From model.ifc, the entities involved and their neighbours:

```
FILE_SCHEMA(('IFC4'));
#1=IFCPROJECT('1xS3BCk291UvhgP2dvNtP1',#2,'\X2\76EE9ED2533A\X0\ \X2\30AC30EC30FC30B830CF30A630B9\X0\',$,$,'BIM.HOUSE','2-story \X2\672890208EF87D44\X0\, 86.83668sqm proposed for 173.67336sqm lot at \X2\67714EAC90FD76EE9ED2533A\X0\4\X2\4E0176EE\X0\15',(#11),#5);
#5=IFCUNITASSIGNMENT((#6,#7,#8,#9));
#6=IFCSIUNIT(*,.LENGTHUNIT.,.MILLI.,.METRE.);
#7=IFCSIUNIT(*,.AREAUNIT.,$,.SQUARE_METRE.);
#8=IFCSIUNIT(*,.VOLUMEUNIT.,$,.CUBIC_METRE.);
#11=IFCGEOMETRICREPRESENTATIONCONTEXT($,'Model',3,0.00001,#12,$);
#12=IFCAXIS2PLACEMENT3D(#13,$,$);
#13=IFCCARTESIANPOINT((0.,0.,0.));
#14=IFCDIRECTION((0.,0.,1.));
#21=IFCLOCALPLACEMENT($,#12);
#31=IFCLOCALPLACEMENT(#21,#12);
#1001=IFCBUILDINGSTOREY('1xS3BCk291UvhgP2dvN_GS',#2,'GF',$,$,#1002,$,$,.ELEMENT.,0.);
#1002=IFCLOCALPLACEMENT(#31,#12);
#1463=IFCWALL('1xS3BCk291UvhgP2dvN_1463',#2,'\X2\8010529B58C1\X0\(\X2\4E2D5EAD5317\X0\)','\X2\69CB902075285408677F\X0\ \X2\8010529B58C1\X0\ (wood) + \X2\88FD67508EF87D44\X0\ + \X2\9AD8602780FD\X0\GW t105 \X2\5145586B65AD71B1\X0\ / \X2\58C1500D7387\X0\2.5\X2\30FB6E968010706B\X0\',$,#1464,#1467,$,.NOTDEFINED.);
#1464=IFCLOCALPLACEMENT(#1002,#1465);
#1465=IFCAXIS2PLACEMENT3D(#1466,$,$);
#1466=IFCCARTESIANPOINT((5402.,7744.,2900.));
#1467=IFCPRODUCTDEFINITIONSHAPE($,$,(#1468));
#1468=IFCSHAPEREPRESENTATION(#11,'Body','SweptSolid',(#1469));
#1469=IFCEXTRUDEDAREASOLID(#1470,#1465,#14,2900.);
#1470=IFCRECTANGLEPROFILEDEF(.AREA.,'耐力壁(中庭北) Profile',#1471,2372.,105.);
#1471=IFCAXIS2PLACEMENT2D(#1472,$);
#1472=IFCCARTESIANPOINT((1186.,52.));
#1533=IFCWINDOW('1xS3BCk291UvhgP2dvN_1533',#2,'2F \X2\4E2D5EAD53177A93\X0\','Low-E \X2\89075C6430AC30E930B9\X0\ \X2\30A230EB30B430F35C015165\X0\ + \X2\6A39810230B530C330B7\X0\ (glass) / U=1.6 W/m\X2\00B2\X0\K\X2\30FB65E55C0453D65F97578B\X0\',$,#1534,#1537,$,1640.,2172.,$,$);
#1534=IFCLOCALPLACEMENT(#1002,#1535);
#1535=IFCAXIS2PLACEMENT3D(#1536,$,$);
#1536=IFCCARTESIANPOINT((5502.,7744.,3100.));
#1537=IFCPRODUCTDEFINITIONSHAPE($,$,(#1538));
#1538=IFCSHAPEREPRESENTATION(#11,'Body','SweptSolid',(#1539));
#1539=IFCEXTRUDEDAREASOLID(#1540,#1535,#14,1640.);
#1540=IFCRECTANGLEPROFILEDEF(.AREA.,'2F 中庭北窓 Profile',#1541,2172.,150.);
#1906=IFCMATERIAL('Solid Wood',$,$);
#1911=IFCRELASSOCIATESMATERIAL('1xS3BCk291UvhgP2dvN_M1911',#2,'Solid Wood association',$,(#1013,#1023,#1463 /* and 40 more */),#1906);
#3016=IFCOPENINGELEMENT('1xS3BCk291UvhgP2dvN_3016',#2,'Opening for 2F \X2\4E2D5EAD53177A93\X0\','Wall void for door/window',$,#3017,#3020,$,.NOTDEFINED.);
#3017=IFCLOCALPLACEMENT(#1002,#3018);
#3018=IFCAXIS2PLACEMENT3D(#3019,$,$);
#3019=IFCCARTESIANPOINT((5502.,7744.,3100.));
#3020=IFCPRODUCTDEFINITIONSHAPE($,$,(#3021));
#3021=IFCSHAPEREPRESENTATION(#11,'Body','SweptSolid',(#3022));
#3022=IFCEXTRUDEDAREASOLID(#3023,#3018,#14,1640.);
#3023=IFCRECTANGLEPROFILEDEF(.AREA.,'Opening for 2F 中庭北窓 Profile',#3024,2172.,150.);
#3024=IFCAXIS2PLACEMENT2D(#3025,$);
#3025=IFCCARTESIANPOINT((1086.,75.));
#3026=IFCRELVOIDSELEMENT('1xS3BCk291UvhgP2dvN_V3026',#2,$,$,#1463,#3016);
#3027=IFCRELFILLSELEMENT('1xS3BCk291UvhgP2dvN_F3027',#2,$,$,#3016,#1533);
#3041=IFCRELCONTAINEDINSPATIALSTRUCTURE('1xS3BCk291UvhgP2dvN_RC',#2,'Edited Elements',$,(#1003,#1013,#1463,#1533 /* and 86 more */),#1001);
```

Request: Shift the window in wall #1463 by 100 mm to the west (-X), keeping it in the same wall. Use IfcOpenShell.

```python
import ifcopenshell
import ifcopenshell.api.geometry
import ifcopenshell.util.placement
import ifcopenshell.util.unit

model = ifcopenshell.open("model.ifc")
unit_scale = ifcopenshell.util.unit.calculate_unit_scale(model)

window = model.by_guid("1xS3BCk291UvhgP2dvN_1533")
opening = window.FillsVoids[0].RelatingOpeningElement
wall = opening.VoidsElements[0].RelatingBuildingElement

wall_matrix = ifcopenshell.util.placement.get_local_placement(wall.ObjectPlacement)
shift = wall_matrix[:3, 0] * -0.1 / unit_scale
before = ifcopenshell.util.placement.get_local_placement(window.ObjectPlacement)[:3, 3].copy()

# The window is not placed relative to its opening, so move both.
for product in (opening, window):
    matrix = ifcopenshell.util.placement.get_local_placement(product.ObjectPlacement)
    matrix[:3, 3] += shift
    ifcopenshell.api.geometry.edit_object_placement(model, product=product, matrix=matrix, is_si=False)

after = ifcopenshell.util.placement.get_local_placement(window.ObjectPlacement)[:3, 3]
print("window moved by", (after - before).round(3) + 0.0)

model.write("model_updated.ifc")
```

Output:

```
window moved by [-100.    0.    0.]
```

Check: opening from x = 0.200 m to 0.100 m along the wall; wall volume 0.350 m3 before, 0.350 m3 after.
